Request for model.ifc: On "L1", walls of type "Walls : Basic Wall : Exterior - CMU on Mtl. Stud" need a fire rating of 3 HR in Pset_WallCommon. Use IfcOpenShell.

First a look at what the model holds.

```python
import ifcopenshell
import ifcopenshell.util.element

model = ifcopenshell.open("model.ifc")
print(model.schema)
storey = next(s for s in model.by_type("IfcBuildingStorey") if s.Name == "L1")
walls = [e for e in ifcopenshell.util.element.get_decomposition(storey) if e.is_a("IfcWall")]
seen = {}
for e in walls:
    element_type = ifcopenshell.util.element.get_type(e)
    key = (element_type.Name if element_type != e and element_type else None, ifcopenshell.util.element.get_pset(e, "Pset_WallCommon", "FireRating"))
    seen[key] = seen.get(key, 0) + 1
for (name, value), count in sorted(seen.items(), key=str):
    print(count, "x", name, "|", value)
```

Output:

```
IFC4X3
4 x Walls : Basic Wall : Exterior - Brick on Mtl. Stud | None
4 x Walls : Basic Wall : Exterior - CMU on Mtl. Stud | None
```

```python
import ifcopenshell
import ifcopenshell.api.pset
import ifcopenshell.util.element

model = ifcopenshell.open("model.ifc")

storey = next(s for s in model.by_type("IfcBuildingStorey") if s.Name == "L1")
walls = [e for e in ifcopenshell.util.element.get_decomposition(storey) if e.is_a("IfcWall")]

count = 0
for e in walls:
    element_type = ifcopenshell.util.element.get_type(e)
    if element_type in (None, e) or element_type.Name != "Walls : Basic Wall : Exterior - CMU on Mtl. Stud":
        continue
    # add_pset returns the element's existing set when there is one.
    pset = ifcopenshell.api.pset.add_pset(model, product=e, name="Pset_WallCommon")
    ifcopenshell.api.pset.edit_pset(model, pset=pset, properties={"FireRating": "3 HR"})
    count += 1

print(count, "walls updated")

model.write("model_edited.ifc")
```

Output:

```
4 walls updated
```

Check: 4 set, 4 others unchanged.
